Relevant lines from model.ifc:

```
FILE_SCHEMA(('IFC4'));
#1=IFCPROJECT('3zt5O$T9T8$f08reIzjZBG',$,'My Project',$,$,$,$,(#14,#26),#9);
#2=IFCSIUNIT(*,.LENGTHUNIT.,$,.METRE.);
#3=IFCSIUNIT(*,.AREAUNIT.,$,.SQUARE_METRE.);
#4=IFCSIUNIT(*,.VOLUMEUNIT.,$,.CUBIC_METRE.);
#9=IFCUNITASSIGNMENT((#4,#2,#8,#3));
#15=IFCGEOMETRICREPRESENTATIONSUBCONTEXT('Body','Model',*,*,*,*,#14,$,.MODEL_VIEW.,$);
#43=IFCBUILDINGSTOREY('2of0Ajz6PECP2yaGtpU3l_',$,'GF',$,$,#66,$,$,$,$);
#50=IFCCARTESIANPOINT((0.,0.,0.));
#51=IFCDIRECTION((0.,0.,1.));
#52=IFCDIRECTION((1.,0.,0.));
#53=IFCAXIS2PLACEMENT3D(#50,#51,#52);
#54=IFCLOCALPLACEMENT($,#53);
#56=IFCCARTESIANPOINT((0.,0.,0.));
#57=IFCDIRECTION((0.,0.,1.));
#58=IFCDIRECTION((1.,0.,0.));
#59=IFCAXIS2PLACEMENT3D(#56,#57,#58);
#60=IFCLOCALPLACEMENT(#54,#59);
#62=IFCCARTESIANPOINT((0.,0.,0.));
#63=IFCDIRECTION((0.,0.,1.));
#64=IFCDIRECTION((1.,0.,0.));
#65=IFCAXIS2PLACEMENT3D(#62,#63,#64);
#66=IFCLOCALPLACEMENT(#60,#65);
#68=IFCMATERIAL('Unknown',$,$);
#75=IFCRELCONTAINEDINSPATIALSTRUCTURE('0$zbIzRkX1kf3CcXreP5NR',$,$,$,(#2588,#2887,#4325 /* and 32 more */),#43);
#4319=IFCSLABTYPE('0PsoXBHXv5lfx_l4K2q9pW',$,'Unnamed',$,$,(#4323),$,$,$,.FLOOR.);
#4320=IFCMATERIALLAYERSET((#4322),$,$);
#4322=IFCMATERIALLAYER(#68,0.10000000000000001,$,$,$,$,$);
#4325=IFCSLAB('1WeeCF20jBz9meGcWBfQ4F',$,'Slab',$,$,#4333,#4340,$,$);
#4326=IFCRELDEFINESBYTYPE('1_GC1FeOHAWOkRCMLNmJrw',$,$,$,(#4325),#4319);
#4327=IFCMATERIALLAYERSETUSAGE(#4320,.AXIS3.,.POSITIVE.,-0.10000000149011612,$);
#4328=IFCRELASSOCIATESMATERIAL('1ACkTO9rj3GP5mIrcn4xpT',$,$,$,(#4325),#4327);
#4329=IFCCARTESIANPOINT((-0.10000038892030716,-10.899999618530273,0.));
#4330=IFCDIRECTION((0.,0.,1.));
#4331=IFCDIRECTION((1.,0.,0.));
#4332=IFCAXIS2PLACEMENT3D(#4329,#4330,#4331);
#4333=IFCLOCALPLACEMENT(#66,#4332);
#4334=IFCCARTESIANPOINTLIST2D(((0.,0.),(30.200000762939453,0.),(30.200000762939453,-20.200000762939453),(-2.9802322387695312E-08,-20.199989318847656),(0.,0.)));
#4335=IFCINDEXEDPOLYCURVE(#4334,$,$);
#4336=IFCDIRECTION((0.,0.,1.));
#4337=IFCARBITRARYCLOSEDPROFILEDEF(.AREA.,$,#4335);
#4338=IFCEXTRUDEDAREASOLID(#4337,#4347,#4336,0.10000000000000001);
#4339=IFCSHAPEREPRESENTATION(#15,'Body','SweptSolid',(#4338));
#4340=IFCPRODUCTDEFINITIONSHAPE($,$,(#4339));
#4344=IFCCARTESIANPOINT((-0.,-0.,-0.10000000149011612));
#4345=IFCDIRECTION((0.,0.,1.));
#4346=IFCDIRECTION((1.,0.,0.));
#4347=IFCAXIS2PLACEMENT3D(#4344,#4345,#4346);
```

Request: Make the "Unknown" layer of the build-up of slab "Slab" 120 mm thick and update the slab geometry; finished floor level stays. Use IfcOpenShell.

```python
import ifcopenshell
import ifcopenshell.util.element
import ifcopenshell.util.representation
import ifcopenshell.util.unit

model = ifcopenshell.open("model.ifc")
unit_scale = ifcopenshell.util.unit.calculate_unit_scale(model)

layer_set = model.by_id(4320)
layer = next(l for l in layer_set.MaterialLayers if l.Material and l.Material.Name == "Unknown")
change = 0.12 / unit_scale - layer.LayerThickness
layer.LayerThickness += change

# Geometry does not follow the layer set by itself.
slabs = [e for e in ifcopenshell.util.element.get_elements_by_material(model, layer_set) if e.is_a("IfcSlab")]
for slab in sorted(slabs, key=lambda e: e.id()):
    body = ifcopenshell.util.representation.get_representation(slab, "Model", "Body")
    solid = body.Items[0]
    old_depth = solid.Depth
    solid.Depth += change
    # Extruded upwards: lower the start of the extrusion so the top stays.
    x, y, z = solid.Position.Location.Coordinates
    solid.Position.Location = model.createIfcCartesianPoint((x, y, z - change))
    print(slab.id(), f"{old_depth:g} -> {solid.Depth:g}")

# The layers are counted up from the underside, which has moved.
for usage in {ifcopenshell.util.element.get_material(slab) for slab in slabs}:
    usage.OffsetFromReferenceLine -= change

model.write("model_v2.ifc")
```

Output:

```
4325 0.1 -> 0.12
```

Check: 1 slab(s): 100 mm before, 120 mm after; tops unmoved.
